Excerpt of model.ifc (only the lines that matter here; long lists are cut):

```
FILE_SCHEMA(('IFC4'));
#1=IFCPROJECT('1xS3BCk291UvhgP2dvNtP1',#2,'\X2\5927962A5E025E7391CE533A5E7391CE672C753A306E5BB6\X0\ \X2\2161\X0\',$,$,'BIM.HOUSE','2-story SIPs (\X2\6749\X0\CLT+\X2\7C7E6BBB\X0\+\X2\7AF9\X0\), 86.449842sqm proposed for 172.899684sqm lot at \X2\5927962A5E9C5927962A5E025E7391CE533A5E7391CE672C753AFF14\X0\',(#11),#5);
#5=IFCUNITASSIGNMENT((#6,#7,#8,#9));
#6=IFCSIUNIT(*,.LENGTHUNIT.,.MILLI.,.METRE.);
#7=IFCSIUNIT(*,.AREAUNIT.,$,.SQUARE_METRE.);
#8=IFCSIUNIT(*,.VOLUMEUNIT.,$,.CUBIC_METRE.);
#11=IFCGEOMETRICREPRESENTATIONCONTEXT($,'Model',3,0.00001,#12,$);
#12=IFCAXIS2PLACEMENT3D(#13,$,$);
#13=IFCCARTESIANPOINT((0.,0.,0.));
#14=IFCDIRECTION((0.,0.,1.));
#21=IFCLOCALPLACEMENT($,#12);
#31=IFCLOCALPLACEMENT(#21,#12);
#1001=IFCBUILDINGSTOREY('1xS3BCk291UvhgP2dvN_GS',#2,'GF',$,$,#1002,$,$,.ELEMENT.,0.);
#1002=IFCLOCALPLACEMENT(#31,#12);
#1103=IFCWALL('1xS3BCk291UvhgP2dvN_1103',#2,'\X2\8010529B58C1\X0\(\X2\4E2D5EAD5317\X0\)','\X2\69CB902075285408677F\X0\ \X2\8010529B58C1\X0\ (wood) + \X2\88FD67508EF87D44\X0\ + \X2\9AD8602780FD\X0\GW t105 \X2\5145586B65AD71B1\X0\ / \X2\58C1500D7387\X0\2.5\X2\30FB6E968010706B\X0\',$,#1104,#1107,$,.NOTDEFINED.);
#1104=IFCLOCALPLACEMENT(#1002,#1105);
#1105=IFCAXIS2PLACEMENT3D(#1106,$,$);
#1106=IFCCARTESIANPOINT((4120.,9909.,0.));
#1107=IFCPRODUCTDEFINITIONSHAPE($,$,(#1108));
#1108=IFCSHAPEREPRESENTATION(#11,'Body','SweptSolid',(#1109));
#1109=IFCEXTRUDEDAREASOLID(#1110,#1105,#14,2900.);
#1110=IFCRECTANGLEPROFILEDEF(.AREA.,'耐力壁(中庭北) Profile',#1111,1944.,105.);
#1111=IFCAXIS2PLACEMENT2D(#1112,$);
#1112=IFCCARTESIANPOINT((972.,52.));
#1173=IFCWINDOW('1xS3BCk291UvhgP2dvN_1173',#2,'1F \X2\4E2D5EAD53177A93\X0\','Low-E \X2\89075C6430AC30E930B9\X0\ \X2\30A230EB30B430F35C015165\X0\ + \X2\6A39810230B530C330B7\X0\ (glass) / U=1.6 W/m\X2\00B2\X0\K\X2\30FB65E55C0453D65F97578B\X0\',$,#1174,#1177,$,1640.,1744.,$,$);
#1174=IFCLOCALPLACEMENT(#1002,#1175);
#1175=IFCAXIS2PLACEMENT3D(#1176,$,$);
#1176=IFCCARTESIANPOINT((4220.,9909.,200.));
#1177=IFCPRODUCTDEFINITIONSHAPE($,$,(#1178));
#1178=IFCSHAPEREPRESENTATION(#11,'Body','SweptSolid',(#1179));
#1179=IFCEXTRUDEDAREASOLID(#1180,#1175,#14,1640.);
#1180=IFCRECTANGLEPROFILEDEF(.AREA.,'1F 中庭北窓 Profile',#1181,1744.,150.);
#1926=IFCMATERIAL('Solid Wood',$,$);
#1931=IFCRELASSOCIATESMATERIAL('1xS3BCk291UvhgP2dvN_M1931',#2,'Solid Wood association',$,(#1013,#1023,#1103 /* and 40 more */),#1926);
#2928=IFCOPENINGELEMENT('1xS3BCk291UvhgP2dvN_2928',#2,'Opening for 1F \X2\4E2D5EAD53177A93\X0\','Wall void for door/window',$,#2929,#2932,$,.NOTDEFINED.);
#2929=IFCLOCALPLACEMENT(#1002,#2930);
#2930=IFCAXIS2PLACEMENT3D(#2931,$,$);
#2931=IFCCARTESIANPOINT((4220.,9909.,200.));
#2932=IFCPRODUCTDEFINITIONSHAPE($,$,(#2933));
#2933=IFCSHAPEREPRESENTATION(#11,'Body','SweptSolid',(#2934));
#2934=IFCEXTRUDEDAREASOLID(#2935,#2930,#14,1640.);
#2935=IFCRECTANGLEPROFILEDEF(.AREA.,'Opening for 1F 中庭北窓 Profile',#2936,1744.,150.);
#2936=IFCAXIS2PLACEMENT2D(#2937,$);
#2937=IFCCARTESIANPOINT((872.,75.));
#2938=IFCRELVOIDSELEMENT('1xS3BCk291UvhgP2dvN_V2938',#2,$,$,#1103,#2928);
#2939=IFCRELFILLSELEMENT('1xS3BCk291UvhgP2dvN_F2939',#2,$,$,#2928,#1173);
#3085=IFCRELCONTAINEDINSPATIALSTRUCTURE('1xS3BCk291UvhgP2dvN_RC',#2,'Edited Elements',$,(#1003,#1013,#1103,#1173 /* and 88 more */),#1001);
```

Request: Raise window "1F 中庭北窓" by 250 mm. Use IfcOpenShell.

```python
import numpy as np
import ifcopenshell
import ifcopenshell.api.geometry
import ifcopenshell.util.placement
import ifcopenshell.util.unit

model = ifcopenshell.open("model.ifc")
unit_scale = ifcopenshell.util.unit.calculate_unit_scale(model)

window = model.by_id(1173)
opening = window.FillsVoids[0].RelatingOpeningElement
dz = 0.25 / unit_scale

shift = np.array([0.0, 0.0, dz])
# The window is not placed relative to its opening, so move both.
for product in (opening, window):
    matrix = ifcopenshell.util.placement.get_local_placement(product.ObjectPlacement)
    matrix[:3, 3] += shift
    ifcopenshell.api.geometry.edit_object_placement(model, product=product, matrix=matrix, is_si=False)

print(f"moved by {dz * unit_scale:+.3f} m")

model.write("model_rev.ifc")
```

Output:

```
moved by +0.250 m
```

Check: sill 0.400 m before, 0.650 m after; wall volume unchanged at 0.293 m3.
